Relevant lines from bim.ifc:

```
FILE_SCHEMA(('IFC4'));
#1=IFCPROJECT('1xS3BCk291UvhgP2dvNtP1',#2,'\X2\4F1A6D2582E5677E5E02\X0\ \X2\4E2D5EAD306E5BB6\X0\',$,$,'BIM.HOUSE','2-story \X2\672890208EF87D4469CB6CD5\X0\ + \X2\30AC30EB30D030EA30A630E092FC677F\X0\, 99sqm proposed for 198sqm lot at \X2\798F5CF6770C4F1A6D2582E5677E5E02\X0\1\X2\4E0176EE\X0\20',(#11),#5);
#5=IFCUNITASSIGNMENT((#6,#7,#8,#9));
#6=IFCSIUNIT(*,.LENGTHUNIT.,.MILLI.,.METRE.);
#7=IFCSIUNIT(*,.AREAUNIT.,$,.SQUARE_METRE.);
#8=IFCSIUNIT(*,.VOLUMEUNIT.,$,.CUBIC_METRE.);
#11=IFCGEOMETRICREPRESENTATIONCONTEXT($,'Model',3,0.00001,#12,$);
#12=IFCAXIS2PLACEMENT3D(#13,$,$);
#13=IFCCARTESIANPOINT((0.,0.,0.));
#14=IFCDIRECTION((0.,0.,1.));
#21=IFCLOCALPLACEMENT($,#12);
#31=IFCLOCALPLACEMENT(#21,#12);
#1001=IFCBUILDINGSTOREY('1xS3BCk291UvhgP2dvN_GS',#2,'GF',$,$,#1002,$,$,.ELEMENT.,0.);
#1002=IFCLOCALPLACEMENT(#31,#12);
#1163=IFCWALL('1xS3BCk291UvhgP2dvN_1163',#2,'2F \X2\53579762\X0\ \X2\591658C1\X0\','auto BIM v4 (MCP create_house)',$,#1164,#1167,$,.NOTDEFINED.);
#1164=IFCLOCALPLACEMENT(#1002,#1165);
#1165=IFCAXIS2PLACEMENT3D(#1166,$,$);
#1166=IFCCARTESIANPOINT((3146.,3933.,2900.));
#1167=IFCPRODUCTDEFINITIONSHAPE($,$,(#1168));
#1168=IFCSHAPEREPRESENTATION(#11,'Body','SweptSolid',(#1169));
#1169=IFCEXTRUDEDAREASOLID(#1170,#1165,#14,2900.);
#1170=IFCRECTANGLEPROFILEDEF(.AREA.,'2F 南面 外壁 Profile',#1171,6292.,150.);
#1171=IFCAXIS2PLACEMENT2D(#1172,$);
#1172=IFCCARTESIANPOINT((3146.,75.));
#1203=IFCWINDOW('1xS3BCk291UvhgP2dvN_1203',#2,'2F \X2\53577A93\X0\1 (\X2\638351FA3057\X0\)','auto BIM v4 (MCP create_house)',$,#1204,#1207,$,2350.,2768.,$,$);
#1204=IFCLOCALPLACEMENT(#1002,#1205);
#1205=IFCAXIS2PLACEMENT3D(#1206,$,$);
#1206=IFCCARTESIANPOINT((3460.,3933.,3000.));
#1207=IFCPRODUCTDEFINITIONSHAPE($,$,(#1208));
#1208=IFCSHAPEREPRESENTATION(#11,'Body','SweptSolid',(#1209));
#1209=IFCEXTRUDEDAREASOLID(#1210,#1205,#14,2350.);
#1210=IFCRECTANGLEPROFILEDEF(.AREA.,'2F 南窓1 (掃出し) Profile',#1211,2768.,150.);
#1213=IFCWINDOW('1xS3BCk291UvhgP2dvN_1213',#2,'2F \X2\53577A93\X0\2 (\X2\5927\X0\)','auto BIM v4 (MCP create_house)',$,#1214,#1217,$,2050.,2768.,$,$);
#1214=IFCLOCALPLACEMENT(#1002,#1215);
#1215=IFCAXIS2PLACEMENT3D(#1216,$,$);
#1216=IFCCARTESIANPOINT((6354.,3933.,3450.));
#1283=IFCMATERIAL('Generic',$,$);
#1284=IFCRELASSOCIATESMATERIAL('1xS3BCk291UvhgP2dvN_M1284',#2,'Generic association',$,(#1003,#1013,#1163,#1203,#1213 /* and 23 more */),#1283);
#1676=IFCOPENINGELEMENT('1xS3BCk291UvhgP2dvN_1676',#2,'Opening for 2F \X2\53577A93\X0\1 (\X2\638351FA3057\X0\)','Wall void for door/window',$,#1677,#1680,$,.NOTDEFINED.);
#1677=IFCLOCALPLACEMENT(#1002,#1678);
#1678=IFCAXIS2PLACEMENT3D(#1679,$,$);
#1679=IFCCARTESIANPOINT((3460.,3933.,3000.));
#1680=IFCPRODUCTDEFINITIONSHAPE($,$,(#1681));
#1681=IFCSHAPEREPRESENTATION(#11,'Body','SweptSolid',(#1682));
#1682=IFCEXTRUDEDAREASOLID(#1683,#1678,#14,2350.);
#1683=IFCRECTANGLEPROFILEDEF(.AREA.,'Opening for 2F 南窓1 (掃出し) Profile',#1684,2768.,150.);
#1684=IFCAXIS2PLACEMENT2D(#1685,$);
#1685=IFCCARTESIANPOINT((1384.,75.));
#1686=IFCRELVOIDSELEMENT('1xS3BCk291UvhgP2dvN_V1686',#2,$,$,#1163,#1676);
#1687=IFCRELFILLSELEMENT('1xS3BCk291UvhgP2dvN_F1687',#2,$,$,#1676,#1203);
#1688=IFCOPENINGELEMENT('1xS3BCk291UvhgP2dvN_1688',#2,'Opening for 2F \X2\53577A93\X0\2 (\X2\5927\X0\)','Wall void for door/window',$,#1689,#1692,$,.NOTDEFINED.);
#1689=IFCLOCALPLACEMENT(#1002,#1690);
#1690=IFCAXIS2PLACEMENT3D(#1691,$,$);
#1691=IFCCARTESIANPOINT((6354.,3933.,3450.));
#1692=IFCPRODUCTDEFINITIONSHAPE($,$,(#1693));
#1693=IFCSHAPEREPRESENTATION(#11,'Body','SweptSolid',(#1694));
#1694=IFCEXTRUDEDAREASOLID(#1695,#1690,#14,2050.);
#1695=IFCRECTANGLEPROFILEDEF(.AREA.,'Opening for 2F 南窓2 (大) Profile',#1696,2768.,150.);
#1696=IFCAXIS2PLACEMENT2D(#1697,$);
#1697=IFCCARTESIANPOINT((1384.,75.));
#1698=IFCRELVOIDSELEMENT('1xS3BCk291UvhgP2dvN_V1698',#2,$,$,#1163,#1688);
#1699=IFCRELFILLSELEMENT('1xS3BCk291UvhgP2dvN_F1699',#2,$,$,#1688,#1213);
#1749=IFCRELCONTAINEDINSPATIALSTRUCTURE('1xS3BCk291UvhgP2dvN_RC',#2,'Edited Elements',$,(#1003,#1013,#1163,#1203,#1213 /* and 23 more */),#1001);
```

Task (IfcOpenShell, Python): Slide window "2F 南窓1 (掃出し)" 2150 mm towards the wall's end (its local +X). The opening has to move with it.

```python
import ifcopenshell
import ifcopenshell.api.geometry
import ifcopenshell.util.placement

model = ifcopenshell.open("bim.ifc")

window = model.by_guid("1xS3BCk291UvhgP2dvN_1203")
opening = window.FillsVoids[0].RelatingOpeningElement
wall = opening.VoidsElements[0].RelatingBuildingElement

wall_matrix = ifcopenshell.util.placement.get_local_placement(wall.ObjectPlacement)
shift = wall_matrix[:3, 0] * 2150.0
before = ifcopenshell.util.placement.get_local_placement(window.ObjectPlacement)[:3, 3].copy()

# The window is not placed relative to its opening, so move both.
for product in (opening, window):
    matrix = ifcopenshell.util.placement.get_local_placement(product.ObjectPlacement)
    matrix[:3, 3] += shift
    ifcopenshell.api.geometry.edit_object_placement(model, product=product, matrix=matrix, is_si=False)

after = ifcopenshell.util.placement.get_local_placement(window.ObjectPlacement)[:3, 3]
print("window moved by", (after - before).round(3) + 0.0)

model.write("bim-out.ifc")
```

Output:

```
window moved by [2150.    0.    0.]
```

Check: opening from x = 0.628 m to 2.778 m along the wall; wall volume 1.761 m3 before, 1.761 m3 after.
